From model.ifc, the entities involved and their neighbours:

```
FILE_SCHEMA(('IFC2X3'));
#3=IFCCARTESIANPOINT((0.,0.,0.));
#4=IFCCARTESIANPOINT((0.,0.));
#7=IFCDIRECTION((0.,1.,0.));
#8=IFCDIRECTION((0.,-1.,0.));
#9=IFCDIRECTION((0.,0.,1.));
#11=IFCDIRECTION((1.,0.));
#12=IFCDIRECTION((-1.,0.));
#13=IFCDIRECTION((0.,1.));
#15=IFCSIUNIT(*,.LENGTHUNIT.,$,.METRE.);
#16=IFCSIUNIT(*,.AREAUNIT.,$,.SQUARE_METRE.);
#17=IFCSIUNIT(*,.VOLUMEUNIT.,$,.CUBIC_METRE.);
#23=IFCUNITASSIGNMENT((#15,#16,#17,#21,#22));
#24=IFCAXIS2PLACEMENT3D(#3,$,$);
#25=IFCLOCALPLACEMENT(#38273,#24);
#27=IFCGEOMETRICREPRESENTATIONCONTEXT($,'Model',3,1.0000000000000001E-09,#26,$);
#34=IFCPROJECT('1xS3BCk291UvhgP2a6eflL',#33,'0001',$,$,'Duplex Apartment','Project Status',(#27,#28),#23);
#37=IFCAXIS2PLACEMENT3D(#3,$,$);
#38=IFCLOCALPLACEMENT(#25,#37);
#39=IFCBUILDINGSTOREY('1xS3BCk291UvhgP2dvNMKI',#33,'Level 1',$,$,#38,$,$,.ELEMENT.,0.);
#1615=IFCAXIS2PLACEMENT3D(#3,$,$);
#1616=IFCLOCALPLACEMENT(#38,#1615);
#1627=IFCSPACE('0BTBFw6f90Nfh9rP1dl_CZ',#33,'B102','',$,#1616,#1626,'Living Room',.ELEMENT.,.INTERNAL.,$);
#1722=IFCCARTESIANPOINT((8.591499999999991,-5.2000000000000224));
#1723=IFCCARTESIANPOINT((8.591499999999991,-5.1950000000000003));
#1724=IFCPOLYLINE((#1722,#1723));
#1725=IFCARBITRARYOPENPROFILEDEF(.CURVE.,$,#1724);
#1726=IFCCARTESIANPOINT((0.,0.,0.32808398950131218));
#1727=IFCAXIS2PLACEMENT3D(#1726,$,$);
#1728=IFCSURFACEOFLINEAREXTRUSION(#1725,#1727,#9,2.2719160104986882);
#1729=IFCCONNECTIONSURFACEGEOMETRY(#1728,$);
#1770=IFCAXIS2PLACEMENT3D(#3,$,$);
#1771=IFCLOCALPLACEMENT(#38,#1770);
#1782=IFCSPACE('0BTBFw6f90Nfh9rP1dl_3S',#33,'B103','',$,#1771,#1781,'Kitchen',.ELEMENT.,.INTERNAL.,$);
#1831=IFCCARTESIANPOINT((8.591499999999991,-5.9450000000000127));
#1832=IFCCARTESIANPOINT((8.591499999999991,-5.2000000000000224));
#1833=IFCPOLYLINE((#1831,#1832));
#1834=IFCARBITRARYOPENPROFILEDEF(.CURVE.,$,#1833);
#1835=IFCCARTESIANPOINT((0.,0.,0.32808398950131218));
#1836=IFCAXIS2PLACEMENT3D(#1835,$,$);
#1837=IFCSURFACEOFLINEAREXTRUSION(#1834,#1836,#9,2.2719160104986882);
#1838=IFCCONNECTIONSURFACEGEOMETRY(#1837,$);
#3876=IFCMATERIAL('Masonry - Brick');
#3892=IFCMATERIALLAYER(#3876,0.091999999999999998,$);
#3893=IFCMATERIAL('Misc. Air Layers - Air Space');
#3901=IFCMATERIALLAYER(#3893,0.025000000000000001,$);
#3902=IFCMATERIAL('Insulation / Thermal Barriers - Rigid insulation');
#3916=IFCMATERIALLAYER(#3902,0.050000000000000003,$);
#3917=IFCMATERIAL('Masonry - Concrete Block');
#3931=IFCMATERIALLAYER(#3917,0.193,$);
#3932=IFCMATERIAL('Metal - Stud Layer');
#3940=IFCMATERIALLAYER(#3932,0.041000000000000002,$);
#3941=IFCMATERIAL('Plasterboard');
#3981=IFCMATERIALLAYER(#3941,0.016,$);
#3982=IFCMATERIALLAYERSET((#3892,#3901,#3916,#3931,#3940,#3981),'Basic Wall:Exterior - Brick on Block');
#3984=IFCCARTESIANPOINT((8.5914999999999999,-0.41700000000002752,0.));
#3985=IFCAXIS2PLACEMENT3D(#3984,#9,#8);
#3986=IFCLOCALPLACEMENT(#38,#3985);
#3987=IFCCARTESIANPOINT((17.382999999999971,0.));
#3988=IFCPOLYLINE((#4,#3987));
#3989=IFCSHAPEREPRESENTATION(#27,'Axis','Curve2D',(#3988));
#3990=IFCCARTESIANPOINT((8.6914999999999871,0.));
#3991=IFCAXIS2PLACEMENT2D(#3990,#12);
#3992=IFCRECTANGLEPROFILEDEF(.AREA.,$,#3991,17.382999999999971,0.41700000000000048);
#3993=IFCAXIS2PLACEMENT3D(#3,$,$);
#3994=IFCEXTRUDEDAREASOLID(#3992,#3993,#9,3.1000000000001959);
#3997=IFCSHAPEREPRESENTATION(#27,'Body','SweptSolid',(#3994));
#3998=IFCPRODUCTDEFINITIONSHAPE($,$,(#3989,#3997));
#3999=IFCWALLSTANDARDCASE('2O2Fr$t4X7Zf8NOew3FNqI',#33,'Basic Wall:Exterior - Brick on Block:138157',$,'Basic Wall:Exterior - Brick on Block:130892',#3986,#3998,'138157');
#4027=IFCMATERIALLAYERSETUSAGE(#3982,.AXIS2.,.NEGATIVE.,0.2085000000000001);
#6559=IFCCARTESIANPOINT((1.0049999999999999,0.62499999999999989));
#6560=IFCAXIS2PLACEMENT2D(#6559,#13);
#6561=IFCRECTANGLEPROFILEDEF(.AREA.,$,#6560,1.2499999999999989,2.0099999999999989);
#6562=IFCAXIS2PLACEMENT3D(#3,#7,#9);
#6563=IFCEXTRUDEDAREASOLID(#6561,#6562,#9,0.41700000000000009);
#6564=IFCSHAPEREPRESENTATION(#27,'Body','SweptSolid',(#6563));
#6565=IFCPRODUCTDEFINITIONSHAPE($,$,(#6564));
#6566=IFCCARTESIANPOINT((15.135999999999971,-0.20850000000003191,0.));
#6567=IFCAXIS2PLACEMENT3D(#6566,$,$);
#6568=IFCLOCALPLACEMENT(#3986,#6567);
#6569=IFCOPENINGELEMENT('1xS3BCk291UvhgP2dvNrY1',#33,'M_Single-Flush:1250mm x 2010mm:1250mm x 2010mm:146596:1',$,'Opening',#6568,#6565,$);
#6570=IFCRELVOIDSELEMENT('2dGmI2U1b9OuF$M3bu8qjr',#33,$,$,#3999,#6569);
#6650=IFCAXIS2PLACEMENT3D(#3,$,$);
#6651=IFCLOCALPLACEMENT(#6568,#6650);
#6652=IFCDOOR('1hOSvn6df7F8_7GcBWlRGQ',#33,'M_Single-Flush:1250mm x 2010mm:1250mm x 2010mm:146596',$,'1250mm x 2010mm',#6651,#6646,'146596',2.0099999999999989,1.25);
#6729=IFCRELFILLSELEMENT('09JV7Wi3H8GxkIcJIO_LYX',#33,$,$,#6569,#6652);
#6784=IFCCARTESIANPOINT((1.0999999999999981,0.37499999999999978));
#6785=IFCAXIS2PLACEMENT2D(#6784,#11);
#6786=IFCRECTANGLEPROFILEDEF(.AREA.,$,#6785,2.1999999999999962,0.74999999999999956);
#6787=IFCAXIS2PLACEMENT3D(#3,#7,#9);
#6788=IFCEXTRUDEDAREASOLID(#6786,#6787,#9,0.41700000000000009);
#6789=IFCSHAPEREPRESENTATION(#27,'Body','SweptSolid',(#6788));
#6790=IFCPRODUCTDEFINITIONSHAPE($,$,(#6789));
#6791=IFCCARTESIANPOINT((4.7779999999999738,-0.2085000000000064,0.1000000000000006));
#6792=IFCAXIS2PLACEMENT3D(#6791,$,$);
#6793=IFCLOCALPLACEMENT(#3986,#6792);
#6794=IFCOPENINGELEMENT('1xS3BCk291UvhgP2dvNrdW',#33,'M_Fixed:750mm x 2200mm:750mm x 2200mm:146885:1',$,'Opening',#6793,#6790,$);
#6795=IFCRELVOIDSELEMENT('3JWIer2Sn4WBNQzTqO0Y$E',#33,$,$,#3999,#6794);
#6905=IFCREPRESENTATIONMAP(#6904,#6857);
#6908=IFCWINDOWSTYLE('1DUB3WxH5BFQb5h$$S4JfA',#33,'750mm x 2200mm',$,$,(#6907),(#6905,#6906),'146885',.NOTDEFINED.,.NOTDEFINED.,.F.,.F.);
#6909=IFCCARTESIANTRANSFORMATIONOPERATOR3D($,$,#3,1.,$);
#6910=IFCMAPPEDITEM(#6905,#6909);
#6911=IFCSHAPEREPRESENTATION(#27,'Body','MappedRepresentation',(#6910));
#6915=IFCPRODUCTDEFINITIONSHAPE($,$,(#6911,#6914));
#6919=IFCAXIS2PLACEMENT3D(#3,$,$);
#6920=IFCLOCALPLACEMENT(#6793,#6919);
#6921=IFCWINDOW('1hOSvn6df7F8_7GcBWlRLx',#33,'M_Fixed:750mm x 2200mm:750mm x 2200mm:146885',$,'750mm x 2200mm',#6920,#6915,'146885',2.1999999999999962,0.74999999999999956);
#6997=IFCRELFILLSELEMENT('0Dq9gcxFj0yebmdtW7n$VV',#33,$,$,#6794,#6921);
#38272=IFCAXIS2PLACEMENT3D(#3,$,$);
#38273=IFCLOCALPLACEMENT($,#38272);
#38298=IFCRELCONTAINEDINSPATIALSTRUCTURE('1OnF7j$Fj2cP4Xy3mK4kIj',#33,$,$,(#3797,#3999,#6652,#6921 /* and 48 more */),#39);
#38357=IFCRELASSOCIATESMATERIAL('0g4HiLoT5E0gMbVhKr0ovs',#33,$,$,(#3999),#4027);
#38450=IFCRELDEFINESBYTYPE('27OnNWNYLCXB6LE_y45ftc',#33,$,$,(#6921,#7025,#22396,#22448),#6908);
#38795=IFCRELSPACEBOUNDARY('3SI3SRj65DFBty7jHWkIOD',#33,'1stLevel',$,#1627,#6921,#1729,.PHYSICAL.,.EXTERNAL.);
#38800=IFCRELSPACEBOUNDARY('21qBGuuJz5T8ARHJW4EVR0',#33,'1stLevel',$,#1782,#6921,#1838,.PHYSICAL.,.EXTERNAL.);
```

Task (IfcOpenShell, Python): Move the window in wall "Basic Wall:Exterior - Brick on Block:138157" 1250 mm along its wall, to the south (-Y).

```python
import numpy as np
import ifcopenshell
import ifcopenshell.api.geometry
import ifcopenshell.util.placement
import ifcopenshell.util.unit

model = ifcopenshell.open("model.ifc")
unit_scale = ifcopenshell.util.unit.calculate_unit_scale(model)

window = model.by_id(6921)
opening = window.FillsVoids[0].RelatingOpeningElement
wall = opening.VoidsElements[0].RelatingBuildingElement

wall_matrix = ifcopenshell.util.placement.get_local_placement(wall.ObjectPlacement)
shift = wall_matrix[:3, 0] * 1.25 / unit_scale
before = ifcopenshell.util.placement.get_local_placement(window.ObjectPlacement)[:3, 3].copy()

# The window is placed relative to its opening, so it follows when the opening moves.
matrix = ifcopenshell.util.placement.get_local_placement(opening.ObjectPlacement)
matrix[:3, 3] += shift
ifcopenshell.api.geometry.edit_object_placement(
    model, product=opening, matrix=matrix, is_si=False, should_transform_children=True
)

# Space boundary surfaces are stored in each space's coordinates; move them too.
for rel in window.ProvidesBoundaries:
    if not rel.ConnectionGeometry:
        continue
    surface = rel.ConnectionGeometry.SurfaceOnRelatingElement
    space_matrix = ifcopenshell.util.placement.get_local_placement(rel.RelatingSpace.ObjectPlacement)
    point = np.array(surface.Position.Location.Coordinates) + space_matrix[:3, :3].T @ shift
    surface.Position = model.createIfcAxis2Placement3D(
        model.createIfcCartesianPoint(point.tolist()), surface.Position.Axis, surface.Position.RefDirection
    )

after = ifcopenshell.util.placement.get_local_placement(window.ObjectPlacement)[:3, 3]
print("window moved by", (after - before).round(3) + 0.0)

model.write("model_v2.ifc")
```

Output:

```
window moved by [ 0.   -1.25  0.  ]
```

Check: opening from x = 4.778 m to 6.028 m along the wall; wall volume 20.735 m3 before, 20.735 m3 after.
